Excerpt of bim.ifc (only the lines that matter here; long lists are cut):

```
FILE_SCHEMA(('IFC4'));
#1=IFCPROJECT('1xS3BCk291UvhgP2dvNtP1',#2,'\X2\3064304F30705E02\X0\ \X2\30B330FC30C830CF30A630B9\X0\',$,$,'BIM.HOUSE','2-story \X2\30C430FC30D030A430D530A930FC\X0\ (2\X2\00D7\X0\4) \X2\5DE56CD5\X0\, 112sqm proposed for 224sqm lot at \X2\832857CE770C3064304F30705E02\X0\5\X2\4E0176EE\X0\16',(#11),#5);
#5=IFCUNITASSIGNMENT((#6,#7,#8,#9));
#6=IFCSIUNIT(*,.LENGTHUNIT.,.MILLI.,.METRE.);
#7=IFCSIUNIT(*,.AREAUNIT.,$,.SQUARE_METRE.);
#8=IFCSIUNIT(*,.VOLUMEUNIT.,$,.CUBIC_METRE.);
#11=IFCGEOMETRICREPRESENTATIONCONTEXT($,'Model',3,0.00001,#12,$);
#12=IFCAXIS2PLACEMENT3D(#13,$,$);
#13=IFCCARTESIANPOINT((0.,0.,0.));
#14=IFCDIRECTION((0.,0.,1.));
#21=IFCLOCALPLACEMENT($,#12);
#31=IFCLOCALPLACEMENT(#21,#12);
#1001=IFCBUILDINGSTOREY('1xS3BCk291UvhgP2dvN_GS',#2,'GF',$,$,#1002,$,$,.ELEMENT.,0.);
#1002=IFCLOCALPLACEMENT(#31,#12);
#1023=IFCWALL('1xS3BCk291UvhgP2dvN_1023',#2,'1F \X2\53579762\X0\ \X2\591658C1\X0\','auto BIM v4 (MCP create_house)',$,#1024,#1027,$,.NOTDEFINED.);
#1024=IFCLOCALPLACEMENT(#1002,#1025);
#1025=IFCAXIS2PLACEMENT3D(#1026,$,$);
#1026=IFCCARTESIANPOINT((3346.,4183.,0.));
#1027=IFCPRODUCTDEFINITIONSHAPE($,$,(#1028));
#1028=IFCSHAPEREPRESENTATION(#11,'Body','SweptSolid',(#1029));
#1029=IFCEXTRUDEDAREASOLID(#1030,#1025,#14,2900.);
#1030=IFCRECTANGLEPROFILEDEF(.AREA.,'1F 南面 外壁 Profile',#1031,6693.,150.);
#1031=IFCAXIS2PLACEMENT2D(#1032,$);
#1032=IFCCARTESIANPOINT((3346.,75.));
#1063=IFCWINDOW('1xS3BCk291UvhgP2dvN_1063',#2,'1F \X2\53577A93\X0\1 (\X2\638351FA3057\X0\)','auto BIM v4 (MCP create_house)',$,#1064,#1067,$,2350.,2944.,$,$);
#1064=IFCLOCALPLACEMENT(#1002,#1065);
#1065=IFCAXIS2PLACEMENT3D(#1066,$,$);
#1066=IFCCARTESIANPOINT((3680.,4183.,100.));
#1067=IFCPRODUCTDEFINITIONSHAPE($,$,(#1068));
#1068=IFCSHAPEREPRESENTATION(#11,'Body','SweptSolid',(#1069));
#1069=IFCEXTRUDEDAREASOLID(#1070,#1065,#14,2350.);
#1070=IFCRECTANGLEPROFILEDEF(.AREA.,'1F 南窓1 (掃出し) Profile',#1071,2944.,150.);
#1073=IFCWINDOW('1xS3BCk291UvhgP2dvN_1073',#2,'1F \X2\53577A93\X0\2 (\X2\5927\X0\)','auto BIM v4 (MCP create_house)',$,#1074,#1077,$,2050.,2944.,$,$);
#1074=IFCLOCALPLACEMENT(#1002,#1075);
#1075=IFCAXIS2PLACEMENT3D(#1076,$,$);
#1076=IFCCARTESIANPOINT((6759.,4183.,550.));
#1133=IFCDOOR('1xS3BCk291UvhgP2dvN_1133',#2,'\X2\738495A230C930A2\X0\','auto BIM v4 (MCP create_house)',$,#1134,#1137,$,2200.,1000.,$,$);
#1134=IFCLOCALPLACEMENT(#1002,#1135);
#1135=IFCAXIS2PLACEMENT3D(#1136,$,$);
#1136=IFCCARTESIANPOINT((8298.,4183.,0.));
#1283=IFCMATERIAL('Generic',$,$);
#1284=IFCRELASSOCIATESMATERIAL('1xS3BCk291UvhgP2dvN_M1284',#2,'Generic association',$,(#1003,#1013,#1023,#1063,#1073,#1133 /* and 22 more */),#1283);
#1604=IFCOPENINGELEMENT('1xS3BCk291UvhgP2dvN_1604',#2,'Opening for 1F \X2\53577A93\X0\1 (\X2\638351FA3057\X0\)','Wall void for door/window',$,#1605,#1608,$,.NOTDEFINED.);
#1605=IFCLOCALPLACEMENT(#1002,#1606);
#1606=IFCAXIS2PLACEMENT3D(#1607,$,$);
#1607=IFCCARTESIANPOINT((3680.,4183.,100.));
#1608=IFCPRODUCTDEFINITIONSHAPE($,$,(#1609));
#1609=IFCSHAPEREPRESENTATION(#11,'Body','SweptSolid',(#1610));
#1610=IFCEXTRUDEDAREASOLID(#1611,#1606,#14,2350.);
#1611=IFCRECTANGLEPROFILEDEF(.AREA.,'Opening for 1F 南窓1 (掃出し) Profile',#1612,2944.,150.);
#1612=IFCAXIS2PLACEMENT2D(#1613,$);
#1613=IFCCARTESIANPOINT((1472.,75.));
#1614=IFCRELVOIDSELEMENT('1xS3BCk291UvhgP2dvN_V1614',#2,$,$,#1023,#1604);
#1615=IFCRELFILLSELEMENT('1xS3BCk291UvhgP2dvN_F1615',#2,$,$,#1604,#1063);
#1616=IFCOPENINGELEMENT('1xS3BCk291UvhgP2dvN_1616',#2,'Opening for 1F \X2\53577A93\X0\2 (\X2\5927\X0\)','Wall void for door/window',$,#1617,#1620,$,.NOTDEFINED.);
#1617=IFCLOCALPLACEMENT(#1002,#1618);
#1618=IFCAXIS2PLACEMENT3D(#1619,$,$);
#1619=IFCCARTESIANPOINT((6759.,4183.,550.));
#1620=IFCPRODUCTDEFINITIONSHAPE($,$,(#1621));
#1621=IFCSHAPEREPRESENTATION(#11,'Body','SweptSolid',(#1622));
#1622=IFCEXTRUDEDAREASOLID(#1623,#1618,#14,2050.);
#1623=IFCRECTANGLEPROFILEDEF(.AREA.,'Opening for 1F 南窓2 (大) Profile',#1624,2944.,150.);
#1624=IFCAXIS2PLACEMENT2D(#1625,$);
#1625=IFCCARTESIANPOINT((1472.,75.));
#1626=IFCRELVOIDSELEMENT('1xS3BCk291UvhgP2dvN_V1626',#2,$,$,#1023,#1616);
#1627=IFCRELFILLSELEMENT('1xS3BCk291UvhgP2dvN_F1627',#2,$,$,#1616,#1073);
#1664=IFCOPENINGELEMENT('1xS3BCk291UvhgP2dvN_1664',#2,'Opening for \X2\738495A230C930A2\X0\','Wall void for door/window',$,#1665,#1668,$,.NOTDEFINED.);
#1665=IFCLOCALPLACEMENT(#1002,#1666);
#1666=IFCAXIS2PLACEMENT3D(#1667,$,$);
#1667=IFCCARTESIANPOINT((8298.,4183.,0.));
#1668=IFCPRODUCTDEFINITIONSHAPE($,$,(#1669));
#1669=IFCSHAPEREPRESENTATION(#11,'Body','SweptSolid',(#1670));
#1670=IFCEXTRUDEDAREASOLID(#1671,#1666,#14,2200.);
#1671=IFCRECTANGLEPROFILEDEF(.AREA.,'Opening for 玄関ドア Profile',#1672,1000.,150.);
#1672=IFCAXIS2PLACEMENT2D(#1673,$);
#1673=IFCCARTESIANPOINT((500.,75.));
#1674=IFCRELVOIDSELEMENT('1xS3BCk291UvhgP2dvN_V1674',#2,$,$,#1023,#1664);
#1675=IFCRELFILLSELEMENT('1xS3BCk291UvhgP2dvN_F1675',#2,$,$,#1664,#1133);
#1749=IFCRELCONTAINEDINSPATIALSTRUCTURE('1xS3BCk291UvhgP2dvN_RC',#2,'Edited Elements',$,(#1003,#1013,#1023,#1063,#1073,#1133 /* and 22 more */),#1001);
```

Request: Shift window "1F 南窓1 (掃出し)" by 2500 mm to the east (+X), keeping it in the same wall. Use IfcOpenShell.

```python
import ifcopenshell
import ifcopenshell.api.geometry
import ifcopenshell.util.placement

model = ifcopenshell.open("bim.ifc")

window = model.by_guid("1xS3BCk291UvhgP2dvN_1063")
opening = window.FillsVoids[0].RelatingOpeningElement
wall = opening.VoidsElements[0].RelatingBuildingElement

wall_matrix = ifcopenshell.util.placement.get_local_placement(wall.ObjectPlacement)
shift = wall_matrix[:3, 0] * 2500.0
before = ifcopenshell.util.placement.get_local_placement(window.ObjectPlacement)[:3, 3].copy()

# The window is not placed relative to its opening, so move both.
for product in (opening, window):
    matrix = ifcopenshell.util.placement.get_local_placement(product.ObjectPlacement)
    matrix[:3, 3] += shift
    ifcopenshell.api.geometry.edit_object_placement(model, product=product, matrix=matrix, is_si=False)

after = ifcopenshell.util.placement.get_local_placement(window.ObjectPlacement)[:3, 3]
print("window moved by", (after - before).round(3) + 0.0)

model.write("bim-out.ifc")
```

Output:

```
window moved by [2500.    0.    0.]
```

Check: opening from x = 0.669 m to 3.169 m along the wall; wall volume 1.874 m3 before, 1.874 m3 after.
